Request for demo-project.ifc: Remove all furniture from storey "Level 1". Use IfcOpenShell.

First a look at what the model holds.

```python
import ifcopenshell
import ifcopenshell.util.element

model = ifcopenshell.open("demo-project.ifc")
print(model.schema)
storey = next(s for s in model.by_type("IfcBuildingStorey") if s.Name == "Level 1")
furniture = [e for e in ifcopenshell.util.element.get_decomposition(storey) if e.is_a("IfcFurnishingElement")]
seen = {}
for e in furniture:
    element_type = ifcopenshell.util.element.get_type(e)
    name = element_type.Name if element_type not in (None, e) else None
    seen[name] = seen.get(name, 0) + 1
for name, count in sorted(seen.items(), key=str):
    print(count, "x", name)
```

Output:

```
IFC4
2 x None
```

```python
import ifcopenshell
import ifcopenshell.api.root
import ifcopenshell.util.element

model = ifcopenshell.open("demo-project.ifc")

storey = next(s for s in model.by_type("IfcBuildingStorey") if s.Name == "Level 1")
furniture = [e for e in ifcopenshell.util.element.get_decomposition(storey) if e.is_a("IfcFurnishingElement")]

for e in furniture:
    ifcopenshell.api.root.remove_product(model, product=e)
print(len(furniture), "removed")

model.write("demo-project_updated.ifc")
```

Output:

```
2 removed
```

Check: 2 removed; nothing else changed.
